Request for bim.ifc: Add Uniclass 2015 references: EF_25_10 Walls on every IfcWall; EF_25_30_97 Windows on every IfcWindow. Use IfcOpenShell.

First a look at what the model holds.

```python
import ifcopenshell

model = ifcopenshell.open("bim.ifc")
print(model.schema)
print("classifications:", [c.Name for c in model.by_type("IfcClassification")])
for ifc_class in ("IfcDoor", "IfcRoof", "IfcStair", "IfcWall", "IfcWindow"):
    print(ifc_class, len(model.by_type(ifc_class)))
```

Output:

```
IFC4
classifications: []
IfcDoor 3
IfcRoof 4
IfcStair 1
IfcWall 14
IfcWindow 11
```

```python
import ifcopenshell
import ifcopenshell.api.classification

model = ifcopenshell.open("bim.ifc")

system = ifcopenshell.api.classification.add_classification(model, classification="Uniclass 2015")

codes = {
    "IfcWall": ("EF_25_10", "Walls"),
    "IfcWindow": ("EF_25_30_97", "Windows"),
}
for ifc_class, (code, name) in codes.items():
    products = model.by_type(ifc_class)
    ifcopenshell.api.classification.add_reference(
        model, products=products, classification=system, identification=code, name=name
    )
    print(code, len(products))

model.write("bim_updated.ifc")
```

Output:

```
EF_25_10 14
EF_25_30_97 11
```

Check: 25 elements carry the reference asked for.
